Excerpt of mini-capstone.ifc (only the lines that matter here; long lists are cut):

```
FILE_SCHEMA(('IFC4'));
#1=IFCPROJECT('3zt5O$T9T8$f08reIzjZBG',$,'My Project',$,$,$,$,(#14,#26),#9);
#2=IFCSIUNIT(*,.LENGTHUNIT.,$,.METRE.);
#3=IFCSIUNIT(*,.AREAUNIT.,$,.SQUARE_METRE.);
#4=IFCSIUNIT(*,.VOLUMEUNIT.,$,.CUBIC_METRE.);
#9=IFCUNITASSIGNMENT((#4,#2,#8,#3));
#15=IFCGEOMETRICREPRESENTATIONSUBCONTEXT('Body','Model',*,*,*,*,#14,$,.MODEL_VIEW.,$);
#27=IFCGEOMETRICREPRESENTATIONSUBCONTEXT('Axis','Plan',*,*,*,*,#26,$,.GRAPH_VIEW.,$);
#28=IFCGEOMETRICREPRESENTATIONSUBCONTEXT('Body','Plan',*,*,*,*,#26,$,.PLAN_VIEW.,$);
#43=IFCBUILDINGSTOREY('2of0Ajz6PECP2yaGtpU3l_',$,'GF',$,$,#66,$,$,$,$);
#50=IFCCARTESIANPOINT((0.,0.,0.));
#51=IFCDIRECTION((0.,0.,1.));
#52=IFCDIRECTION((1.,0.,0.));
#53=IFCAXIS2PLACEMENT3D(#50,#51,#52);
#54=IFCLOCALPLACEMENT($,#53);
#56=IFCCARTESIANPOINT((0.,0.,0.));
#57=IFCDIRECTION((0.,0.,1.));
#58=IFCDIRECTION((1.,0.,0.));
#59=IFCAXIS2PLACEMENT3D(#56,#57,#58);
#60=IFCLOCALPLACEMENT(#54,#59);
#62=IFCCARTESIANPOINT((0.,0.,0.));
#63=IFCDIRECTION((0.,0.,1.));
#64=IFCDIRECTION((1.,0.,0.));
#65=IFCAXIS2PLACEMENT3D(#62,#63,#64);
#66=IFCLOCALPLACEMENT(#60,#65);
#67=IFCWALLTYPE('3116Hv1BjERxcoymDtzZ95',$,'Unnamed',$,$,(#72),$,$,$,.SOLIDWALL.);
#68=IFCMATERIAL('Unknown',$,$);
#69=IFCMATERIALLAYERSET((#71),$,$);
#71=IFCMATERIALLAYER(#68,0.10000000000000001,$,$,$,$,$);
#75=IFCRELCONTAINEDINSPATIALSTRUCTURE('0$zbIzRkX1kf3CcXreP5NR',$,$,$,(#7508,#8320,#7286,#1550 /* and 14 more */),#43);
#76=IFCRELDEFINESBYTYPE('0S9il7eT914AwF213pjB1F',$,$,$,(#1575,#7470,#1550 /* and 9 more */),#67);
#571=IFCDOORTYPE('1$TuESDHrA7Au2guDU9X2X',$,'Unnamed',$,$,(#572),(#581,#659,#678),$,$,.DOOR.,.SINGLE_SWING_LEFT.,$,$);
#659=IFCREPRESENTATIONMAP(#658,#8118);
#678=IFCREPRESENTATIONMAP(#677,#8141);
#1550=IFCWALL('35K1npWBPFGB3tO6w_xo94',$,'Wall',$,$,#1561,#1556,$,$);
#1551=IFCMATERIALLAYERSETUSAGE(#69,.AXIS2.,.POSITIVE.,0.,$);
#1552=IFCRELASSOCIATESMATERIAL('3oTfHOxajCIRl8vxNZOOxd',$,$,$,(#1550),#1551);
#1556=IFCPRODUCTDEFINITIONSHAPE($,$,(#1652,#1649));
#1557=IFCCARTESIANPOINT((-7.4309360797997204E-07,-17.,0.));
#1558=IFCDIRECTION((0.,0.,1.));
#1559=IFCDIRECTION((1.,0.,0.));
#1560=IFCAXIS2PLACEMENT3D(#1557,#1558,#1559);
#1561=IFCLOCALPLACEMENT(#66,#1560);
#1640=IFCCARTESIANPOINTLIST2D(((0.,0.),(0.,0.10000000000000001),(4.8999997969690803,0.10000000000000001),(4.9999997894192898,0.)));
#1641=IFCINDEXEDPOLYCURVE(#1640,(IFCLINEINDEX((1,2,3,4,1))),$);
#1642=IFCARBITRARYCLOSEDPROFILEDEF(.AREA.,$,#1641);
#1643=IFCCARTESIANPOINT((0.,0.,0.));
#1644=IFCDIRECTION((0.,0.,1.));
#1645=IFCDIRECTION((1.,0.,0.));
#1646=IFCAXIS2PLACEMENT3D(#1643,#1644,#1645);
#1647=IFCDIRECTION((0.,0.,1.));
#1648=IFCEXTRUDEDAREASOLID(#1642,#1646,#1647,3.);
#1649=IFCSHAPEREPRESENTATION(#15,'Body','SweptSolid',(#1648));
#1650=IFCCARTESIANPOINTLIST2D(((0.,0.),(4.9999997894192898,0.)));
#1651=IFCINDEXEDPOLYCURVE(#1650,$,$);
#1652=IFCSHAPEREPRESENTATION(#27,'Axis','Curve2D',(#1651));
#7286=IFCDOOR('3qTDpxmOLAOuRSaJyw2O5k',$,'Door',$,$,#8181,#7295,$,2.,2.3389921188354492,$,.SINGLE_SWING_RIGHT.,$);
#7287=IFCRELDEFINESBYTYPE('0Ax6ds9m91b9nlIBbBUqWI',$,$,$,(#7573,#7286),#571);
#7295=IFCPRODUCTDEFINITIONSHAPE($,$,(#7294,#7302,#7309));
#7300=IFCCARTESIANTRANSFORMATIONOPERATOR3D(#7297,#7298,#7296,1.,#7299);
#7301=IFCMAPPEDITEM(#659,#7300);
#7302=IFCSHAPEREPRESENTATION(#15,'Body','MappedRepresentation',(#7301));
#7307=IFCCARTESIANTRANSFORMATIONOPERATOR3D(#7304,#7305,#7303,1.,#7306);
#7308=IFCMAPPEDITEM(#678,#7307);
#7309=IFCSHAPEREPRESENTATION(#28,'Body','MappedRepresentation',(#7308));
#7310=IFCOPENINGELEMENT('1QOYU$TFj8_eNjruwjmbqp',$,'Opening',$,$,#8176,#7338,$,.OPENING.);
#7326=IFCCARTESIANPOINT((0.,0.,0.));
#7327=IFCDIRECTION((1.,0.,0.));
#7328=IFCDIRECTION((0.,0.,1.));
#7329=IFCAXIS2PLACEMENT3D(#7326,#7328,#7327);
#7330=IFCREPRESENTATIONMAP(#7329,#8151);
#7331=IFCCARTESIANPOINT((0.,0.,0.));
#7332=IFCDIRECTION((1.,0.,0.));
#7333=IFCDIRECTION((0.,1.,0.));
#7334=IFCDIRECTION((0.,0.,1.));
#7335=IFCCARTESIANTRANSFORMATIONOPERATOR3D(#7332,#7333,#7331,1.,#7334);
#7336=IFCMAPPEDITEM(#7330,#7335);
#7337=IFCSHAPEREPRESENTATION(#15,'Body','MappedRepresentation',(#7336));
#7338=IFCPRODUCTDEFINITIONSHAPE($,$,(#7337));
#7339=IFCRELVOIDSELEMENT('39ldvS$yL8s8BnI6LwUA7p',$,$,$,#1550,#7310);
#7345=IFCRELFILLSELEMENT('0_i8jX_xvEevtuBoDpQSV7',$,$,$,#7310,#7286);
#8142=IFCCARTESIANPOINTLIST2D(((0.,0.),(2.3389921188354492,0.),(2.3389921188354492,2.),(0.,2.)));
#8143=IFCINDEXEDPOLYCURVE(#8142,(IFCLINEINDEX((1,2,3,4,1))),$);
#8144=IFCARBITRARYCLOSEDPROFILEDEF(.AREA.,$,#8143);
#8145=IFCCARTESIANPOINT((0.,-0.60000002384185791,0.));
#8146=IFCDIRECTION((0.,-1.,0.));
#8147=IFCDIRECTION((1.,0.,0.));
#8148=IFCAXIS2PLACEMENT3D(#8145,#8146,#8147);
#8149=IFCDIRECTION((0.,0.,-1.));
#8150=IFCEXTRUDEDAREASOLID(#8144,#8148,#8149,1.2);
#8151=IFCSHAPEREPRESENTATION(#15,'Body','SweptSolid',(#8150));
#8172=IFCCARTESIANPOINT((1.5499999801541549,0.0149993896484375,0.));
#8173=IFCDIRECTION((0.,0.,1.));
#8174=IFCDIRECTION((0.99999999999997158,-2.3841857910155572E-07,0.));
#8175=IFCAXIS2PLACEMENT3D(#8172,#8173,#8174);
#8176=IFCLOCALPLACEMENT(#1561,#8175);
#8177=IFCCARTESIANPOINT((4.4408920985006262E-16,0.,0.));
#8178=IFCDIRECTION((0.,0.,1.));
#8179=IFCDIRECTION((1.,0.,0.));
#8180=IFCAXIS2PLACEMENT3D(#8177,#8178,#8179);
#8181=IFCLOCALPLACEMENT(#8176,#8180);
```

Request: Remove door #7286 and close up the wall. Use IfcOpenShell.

```python
import ifcopenshell
import ifcopenshell.api.feature
import ifcopenshell.api.root
import ifcopenshell.geom
import ifcopenshell.util.shape

model = ifcopenshell.open("mini-capstone.ifc")
settings = ifcopenshell.geom.settings()


def volume(element):
    """Net volume in cubic metres, openings subtracted."""
    shape = ifcopenshell.geom.create_shape(settings, element)
    return ifcopenshell.util.shape.get_volume(shape.geometry)


door = model.by_guid("3qTDpxmOLAOuRSaJyw2O5k")
opening = door.FillsVoids[0].RelatingOpeningElement
wall = opening.VoidsElements[0].RelatingBuildingElement
before = volume(wall)

ifcopenshell.api.root.remove_product(model, product=door)
ifcopenshell.api.feature.remove_feature(model, feature=opening)

after = volume(wall)

print(f"wall volume {before:.3f} -> {after:.3f} m3")

model.write("mini-capstone-out.ifc")
```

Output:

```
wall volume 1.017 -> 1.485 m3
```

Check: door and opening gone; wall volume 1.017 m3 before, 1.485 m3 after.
